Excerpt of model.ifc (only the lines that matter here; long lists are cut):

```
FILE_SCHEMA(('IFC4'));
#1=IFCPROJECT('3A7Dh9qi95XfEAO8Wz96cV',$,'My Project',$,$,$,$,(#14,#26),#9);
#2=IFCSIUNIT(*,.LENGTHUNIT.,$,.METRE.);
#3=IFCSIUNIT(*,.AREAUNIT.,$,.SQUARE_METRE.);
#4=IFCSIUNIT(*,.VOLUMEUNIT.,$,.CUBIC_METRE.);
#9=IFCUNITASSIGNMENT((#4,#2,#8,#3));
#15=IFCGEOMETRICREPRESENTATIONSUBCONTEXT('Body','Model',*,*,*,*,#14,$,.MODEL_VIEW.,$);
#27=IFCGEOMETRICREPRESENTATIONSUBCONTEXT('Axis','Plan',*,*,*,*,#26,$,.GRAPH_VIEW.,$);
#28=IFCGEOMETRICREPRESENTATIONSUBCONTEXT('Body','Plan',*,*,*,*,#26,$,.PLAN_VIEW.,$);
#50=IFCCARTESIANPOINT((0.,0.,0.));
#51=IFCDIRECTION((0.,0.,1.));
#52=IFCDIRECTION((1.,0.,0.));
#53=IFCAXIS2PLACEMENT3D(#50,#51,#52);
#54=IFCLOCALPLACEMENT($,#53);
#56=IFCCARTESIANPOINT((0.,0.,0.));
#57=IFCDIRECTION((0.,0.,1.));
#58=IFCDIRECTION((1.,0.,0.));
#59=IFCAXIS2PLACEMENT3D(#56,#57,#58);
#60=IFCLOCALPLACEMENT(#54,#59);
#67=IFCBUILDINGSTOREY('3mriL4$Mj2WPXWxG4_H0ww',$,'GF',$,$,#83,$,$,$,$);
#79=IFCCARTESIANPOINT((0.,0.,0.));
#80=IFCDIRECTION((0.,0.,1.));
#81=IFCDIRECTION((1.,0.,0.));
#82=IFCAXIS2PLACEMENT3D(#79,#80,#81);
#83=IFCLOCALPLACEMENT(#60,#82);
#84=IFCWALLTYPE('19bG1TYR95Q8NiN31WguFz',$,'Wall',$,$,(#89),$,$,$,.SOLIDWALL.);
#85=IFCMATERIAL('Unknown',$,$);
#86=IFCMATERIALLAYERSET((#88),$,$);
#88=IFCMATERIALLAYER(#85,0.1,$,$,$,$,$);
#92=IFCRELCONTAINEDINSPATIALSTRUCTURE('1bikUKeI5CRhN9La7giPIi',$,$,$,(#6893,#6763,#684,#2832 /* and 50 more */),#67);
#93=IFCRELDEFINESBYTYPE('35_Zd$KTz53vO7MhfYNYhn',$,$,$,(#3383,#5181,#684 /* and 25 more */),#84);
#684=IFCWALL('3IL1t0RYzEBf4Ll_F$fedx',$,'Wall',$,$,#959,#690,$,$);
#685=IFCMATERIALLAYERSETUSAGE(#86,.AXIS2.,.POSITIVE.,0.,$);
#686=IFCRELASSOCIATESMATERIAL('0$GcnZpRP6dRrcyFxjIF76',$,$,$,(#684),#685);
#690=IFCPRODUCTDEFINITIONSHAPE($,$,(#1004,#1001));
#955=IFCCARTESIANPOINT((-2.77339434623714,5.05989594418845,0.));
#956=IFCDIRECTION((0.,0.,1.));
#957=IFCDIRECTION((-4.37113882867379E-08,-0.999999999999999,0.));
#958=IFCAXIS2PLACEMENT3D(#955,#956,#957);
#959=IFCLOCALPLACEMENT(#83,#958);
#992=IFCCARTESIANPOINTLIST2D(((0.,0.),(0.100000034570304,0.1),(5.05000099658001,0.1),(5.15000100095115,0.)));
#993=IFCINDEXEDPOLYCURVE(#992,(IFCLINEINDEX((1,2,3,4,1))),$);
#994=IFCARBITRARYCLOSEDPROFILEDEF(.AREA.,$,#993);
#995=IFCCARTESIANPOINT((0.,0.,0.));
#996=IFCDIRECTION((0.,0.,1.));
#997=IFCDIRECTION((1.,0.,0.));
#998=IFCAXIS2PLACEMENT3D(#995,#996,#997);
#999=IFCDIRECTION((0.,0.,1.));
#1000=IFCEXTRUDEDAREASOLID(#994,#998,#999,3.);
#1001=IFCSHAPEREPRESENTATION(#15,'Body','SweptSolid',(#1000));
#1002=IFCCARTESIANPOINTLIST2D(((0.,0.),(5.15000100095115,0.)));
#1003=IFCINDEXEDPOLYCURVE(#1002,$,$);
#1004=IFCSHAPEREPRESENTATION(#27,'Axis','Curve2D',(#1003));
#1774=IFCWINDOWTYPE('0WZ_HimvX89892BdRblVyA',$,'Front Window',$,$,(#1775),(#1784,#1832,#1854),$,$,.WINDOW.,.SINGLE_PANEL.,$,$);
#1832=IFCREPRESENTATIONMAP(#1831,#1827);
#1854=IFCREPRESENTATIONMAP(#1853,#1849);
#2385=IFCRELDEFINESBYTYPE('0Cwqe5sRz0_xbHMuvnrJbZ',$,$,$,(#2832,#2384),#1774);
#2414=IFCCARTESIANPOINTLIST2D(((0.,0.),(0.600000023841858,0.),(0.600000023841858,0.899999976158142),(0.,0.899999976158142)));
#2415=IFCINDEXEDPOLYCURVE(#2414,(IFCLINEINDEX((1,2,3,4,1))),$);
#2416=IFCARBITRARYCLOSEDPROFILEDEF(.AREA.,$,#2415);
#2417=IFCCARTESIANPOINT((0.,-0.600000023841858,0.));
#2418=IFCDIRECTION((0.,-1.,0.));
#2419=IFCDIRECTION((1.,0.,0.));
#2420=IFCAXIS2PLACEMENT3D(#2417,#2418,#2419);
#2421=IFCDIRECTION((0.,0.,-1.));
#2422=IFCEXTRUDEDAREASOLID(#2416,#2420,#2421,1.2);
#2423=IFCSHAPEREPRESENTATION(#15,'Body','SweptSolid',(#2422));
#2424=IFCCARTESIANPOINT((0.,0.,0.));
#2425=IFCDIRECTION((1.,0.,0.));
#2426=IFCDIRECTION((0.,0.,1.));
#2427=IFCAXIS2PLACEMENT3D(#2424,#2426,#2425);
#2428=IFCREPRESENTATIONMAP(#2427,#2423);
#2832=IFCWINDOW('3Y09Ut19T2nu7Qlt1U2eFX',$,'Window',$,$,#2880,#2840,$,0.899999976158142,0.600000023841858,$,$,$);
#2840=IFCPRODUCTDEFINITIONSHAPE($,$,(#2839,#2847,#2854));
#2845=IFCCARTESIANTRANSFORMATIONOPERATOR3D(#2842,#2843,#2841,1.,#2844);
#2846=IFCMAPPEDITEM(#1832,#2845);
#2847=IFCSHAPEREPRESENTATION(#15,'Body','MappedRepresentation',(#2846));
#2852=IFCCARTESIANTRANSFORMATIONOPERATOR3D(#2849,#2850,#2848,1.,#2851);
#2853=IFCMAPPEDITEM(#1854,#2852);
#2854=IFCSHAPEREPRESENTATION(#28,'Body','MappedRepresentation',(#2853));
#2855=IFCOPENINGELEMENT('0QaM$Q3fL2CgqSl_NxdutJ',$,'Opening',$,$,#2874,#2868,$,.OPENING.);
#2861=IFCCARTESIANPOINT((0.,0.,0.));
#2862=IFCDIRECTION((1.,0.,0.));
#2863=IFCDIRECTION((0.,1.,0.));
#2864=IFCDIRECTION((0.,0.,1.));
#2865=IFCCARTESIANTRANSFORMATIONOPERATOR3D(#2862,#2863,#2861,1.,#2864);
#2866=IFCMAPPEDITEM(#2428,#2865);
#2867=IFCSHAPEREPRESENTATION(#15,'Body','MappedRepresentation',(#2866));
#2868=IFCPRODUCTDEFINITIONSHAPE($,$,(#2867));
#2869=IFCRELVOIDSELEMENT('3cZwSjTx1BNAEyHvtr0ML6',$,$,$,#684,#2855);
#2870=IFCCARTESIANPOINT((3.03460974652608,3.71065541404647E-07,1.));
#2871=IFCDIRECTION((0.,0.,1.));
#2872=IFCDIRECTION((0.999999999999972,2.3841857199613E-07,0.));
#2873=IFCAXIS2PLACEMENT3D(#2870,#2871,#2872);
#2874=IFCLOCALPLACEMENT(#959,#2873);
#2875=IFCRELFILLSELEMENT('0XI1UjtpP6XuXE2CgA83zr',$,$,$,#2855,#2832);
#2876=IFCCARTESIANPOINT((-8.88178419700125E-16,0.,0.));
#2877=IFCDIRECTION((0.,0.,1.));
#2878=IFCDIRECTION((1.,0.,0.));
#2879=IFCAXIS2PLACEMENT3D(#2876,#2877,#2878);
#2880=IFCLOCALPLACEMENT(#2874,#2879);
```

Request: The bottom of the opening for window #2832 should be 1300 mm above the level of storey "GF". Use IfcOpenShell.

```python
import numpy as np
import ifcopenshell
import ifcopenshell.api.geometry
import ifcopenshell.geom
import ifcopenshell.util.element
import ifcopenshell.util.placement
import ifcopenshell.util.shape
import ifcopenshell.util.unit

model = ifcopenshell.open("model.ifc")
unit_scale = ifcopenshell.util.unit.calculate_unit_scale(model)

window = model.by_guid("3Y09Ut19T2nu7Qlt1U2eFX")
opening = window.FillsVoids[0].RelatingOpeningElement
storey = ifcopenshell.util.element.get_container(window, ifc_class="IfcBuildingStorey")
level = ifcopenshell.util.placement.get_local_placement(storey.ObjectPlacement)[2, 3]

# The opening's origin need not be at the sill, so measure its lowest point.
shape = ifcopenshell.geom.create_shape(ifcopenshell.geom.settings(), opening)
bottom = ifcopenshell.util.shape.get_shape_bottom_elevation(shape, shape.geometry) / unit_scale
dz = level + 1.3 / unit_scale - bottom

shift = np.array([0.0, 0.0, dz])
# The window is placed relative to its opening, so it follows when the opening moves.
matrix = ifcopenshell.util.placement.get_local_placement(opening.ObjectPlacement)
matrix[:3, 3] += shift
ifcopenshell.api.geometry.edit_object_placement(
    model, product=opening, matrix=matrix, is_si=False, should_transform_children=True
)

print(f"moved by {dz * unit_scale:+.3f} m")

model.write("model_rev.ifc")
```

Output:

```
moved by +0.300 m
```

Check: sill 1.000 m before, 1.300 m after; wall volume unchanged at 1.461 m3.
